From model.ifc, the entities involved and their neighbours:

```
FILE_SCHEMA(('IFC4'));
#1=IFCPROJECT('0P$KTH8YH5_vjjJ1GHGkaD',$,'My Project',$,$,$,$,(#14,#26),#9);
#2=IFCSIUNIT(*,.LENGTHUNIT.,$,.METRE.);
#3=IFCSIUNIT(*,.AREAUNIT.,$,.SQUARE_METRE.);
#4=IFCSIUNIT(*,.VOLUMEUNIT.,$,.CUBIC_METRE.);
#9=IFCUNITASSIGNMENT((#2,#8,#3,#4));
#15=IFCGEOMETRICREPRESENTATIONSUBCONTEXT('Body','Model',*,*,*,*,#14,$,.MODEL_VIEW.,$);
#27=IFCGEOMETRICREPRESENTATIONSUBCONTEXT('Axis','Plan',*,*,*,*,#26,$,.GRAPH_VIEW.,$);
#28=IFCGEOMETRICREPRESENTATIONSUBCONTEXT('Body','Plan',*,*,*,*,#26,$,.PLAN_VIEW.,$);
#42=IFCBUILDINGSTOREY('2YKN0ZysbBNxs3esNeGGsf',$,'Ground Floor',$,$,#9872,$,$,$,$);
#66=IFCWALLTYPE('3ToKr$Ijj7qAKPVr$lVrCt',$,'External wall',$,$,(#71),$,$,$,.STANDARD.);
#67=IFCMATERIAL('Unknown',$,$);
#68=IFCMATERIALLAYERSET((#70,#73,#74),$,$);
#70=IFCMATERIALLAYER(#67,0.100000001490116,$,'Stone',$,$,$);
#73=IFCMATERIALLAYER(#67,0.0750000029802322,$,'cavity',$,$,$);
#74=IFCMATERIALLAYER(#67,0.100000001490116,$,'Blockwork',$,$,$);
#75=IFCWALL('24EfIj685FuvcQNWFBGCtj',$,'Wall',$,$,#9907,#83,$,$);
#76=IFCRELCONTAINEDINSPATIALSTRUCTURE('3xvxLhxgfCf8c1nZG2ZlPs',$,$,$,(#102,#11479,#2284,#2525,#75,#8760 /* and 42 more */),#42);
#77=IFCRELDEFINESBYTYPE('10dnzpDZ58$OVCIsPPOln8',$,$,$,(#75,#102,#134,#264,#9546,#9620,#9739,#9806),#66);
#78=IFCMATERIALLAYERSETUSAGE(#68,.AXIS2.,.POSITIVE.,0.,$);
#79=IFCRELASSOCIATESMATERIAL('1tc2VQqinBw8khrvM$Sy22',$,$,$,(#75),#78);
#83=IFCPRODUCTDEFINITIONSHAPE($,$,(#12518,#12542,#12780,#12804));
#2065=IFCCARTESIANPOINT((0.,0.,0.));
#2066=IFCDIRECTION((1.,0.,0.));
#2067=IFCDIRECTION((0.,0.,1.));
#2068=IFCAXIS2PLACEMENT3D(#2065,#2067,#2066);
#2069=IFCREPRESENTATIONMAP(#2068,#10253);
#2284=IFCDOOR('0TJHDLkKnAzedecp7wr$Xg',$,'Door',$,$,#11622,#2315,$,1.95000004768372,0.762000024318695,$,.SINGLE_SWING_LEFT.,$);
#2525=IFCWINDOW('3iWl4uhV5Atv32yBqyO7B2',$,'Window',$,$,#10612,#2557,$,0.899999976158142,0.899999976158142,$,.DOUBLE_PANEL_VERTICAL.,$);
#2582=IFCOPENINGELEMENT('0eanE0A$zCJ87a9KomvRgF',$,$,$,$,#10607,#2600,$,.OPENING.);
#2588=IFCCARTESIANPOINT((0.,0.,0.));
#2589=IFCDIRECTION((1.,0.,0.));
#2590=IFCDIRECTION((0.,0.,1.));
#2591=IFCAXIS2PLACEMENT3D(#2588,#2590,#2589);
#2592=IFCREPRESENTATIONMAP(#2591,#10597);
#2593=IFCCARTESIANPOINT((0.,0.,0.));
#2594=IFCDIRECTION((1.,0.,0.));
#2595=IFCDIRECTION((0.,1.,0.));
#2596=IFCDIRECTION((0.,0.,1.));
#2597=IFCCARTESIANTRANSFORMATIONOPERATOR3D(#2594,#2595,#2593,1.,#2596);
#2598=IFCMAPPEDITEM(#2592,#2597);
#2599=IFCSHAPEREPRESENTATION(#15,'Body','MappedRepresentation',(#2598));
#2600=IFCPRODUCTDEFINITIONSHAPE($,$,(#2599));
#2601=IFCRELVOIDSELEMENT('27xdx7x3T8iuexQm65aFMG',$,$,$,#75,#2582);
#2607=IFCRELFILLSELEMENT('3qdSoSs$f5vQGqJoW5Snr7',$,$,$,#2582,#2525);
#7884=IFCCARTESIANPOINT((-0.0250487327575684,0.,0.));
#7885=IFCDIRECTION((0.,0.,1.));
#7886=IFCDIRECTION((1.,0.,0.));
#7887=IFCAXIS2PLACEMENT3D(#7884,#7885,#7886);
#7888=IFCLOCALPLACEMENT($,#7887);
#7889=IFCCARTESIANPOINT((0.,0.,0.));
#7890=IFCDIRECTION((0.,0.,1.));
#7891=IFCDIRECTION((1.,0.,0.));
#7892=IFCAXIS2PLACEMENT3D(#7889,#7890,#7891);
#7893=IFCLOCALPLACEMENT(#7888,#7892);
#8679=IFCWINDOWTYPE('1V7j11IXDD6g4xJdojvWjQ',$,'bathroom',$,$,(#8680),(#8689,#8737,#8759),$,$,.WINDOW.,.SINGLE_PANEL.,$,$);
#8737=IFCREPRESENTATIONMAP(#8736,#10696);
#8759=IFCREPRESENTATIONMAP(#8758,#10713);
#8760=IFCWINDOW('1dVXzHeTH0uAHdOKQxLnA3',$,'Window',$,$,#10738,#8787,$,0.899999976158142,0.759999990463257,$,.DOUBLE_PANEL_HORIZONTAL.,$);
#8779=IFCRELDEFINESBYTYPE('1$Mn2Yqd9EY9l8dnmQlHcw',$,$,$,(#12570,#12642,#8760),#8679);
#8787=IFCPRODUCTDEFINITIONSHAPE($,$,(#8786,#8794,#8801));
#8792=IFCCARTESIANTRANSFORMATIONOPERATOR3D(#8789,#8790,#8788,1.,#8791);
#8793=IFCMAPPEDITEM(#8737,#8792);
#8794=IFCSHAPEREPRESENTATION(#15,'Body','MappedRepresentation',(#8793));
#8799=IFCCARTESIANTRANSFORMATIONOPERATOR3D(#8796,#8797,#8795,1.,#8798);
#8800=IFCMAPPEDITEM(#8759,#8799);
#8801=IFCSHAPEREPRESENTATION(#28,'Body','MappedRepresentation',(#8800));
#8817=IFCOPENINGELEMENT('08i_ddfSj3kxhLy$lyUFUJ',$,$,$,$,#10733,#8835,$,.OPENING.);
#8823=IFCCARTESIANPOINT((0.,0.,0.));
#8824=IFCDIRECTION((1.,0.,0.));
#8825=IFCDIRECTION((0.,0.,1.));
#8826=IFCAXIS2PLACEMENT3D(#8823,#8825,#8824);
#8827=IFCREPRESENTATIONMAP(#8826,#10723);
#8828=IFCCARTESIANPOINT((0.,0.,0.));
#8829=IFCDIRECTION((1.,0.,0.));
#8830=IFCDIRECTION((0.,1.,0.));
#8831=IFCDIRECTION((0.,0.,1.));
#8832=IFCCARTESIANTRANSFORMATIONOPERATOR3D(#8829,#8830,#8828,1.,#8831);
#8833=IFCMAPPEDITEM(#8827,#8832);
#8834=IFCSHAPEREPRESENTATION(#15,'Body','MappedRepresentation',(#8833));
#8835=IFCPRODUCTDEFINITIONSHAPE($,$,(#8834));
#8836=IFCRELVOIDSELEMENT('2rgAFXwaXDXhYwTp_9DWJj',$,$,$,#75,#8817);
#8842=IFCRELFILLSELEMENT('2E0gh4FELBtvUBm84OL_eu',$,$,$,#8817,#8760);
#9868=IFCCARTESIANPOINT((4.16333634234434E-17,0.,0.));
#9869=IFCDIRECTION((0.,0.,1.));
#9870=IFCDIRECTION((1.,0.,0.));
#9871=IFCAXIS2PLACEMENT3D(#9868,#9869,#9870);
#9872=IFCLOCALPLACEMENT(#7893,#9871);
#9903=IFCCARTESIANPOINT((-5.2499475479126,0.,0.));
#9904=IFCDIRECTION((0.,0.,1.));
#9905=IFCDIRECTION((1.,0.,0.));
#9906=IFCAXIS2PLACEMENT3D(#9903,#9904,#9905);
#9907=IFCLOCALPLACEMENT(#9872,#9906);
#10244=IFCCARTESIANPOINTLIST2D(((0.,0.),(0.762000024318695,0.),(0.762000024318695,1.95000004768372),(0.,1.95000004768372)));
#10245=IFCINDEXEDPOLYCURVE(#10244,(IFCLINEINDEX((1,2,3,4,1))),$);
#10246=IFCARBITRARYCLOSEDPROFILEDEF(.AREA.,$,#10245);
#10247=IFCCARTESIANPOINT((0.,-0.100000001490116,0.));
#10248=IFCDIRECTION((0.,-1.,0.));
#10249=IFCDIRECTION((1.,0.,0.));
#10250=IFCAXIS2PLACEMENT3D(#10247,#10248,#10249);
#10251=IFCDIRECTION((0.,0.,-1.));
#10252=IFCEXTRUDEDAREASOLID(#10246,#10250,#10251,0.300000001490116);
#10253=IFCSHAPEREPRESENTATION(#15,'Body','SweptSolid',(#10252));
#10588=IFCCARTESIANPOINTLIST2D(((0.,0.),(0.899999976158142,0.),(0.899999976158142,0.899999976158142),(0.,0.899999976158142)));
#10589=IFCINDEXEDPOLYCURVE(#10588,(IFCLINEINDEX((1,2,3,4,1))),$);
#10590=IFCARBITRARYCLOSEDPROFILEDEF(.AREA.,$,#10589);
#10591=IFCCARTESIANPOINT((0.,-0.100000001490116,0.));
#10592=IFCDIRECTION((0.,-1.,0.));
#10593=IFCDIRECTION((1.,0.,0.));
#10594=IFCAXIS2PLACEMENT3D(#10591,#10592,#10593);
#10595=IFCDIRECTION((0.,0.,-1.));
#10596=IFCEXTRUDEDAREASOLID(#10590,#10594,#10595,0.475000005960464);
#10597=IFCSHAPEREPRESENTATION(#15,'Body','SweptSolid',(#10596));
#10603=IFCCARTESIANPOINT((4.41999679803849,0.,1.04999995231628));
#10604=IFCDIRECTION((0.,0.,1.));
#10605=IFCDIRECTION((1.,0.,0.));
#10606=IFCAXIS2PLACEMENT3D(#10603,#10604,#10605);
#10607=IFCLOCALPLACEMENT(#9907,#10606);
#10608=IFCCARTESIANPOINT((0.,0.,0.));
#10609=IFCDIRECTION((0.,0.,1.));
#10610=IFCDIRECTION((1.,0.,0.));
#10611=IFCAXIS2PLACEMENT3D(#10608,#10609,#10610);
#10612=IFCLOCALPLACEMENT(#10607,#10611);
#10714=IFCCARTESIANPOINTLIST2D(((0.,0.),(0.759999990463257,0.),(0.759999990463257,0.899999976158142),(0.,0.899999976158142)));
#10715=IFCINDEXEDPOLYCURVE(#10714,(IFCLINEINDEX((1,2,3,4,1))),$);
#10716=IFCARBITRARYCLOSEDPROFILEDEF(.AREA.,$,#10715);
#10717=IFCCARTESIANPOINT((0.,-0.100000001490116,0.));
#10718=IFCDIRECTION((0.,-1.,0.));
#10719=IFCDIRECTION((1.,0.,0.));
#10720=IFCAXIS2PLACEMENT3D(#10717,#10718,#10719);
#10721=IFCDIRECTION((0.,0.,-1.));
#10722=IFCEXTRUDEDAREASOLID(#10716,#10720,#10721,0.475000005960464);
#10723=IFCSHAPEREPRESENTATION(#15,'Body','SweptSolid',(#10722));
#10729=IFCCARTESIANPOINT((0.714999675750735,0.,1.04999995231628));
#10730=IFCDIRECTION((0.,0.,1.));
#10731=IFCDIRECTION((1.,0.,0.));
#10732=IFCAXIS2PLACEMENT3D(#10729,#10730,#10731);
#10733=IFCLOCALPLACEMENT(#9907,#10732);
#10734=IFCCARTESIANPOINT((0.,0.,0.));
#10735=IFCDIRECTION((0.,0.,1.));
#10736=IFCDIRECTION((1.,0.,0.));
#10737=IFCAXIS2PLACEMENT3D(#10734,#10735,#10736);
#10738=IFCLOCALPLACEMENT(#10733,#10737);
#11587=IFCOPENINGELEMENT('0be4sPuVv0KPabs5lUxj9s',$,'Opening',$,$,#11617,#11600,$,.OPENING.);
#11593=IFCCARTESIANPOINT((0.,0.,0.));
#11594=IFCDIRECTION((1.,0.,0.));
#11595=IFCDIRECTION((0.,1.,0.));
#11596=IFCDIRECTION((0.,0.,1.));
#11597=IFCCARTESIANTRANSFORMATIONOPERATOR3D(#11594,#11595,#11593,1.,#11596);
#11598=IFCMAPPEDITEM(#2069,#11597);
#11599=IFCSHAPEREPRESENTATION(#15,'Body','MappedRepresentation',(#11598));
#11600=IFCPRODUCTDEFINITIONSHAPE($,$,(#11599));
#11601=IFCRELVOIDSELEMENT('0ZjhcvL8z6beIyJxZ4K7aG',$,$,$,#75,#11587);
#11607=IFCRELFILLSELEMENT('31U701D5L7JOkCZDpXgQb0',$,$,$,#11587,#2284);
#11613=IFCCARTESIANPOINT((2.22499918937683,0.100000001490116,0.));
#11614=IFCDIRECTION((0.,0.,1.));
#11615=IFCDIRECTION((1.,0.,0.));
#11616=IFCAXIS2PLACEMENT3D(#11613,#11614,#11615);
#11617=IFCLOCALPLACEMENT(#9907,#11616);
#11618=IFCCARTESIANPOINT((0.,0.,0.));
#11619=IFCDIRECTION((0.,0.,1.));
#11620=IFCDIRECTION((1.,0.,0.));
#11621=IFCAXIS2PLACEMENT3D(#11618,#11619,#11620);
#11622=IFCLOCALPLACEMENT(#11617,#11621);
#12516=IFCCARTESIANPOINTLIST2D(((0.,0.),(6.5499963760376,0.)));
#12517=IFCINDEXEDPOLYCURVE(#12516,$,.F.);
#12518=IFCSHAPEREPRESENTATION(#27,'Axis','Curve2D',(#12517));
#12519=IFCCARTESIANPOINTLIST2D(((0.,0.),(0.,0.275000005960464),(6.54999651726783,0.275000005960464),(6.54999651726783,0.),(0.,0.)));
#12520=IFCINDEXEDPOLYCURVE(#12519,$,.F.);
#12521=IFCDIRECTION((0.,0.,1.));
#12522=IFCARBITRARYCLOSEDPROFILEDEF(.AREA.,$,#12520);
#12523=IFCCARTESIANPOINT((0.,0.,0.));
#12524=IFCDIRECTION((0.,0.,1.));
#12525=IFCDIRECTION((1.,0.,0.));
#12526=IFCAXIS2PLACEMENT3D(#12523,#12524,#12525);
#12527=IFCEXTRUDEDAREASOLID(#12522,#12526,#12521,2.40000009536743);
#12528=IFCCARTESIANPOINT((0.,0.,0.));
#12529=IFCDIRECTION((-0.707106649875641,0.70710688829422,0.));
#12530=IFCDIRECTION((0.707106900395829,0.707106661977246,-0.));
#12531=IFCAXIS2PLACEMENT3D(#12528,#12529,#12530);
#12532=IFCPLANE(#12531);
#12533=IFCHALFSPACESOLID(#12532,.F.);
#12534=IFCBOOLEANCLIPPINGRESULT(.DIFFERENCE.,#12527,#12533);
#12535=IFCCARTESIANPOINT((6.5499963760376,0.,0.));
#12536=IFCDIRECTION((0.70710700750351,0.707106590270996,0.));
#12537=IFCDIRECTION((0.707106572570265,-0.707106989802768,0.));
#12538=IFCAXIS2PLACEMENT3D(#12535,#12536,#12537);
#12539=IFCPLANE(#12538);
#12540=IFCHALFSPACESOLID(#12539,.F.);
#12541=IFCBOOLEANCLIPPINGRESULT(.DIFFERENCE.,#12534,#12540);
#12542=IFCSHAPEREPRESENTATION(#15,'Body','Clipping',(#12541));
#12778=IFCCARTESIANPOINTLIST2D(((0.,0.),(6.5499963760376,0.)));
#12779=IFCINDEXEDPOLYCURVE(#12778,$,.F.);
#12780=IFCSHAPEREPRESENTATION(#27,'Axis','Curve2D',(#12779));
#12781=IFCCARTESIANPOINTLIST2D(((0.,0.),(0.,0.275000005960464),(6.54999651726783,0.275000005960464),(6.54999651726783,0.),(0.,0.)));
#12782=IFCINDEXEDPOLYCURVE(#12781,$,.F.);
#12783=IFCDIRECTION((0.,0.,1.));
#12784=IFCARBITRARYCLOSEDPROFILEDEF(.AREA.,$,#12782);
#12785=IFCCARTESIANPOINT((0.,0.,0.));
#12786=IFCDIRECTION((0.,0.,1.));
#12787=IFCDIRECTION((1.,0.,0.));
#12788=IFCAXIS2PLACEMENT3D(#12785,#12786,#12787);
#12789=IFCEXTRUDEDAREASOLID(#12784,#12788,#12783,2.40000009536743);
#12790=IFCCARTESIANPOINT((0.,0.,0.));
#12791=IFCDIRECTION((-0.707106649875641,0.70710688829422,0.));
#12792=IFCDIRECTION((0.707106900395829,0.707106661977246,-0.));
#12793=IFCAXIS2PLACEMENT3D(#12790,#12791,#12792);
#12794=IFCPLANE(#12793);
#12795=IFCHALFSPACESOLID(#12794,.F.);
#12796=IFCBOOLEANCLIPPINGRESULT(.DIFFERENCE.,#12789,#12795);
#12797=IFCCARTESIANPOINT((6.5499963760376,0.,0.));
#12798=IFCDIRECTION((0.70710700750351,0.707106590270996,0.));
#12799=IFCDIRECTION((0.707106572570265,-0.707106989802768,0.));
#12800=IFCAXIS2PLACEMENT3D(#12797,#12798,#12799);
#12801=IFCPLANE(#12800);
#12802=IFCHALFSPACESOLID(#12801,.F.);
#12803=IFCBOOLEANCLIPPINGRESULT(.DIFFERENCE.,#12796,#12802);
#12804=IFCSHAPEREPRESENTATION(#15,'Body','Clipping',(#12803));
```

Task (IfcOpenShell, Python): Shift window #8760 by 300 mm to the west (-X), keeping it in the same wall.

```python
import ifcopenshell
import ifcopenshell.api.geometry
import ifcopenshell.util.placement
import ifcopenshell.util.unit

model = ifcopenshell.open("model.ifc")
unit_scale = ifcopenshell.util.unit.calculate_unit_scale(model)

window = model.by_id(8760)
opening = window.FillsVoids[0].RelatingOpeningElement
wall = opening.VoidsElements[0].RelatingBuildingElement

wall_matrix = ifcopenshell.util.placement.get_local_placement(wall.ObjectPlacement)
shift = wall_matrix[:3, 0] * -0.3 / unit_scale
before = ifcopenshell.util.placement.get_local_placement(window.ObjectPlacement)[:3, 3].copy()

# The window is placed relative to its opening, so it follows when the opening moves.
matrix = ifcopenshell.util.placement.get_local_placement(opening.ObjectPlacement)
matrix[:3, 3] += shift
ifcopenshell.api.geometry.edit_object_placement(
    model, product=opening, matrix=matrix, is_si=False, should_transform_children=True
)

after = ifcopenshell.util.placement.get_local_placement(window.ObjectPlacement)[:3, 3]
print("window moved by", (after - before).round(3) + 0.0)

model.write("model_edited.ifc")
```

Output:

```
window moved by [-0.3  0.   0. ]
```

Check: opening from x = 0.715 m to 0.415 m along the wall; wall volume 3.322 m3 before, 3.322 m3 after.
